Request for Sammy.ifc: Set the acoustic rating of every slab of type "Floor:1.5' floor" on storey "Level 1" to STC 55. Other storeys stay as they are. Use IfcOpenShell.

First a look at what the model holds.

```python
import ifcopenshell
import ifcopenshell.util.element

model = ifcopenshell.open("Sammy.ifc")
print(model.schema)
storey = next(s for s in model.by_type("IfcBuildingStorey") if s.Name == "Level 1")
slabs = [e for e in ifcopenshell.util.element.get_decomposition(storey) if e.is_a("IfcSlab")]
seen = {}
for e in slabs:
    element_type = ifcopenshell.util.element.get_type(e)
    key = (element_type.Name if element_type != e and element_type else None, ifcopenshell.util.element.get_pset(e, "Pset_SlabCommon", "AcousticRating"))
    seen[key] = seen.get(key, 0) + 1
for (name, value), count in sorted(seen.items(), key=str):
    print(count, "x", name, "|", value)
```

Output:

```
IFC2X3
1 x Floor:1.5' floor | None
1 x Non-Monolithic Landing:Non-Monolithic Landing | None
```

```python
import ifcopenshell
import ifcopenshell.api.pset
import ifcopenshell.util.element

model = ifcopenshell.open("Sammy.ifc")

storey = next(s for s in model.by_type("IfcBuildingStorey") if s.Name == "Level 1")
slabs = [e for e in ifcopenshell.util.element.get_decomposition(storey) if e.is_a("IfcSlab")]

count = 0
for e in slabs:
    element_type = ifcopenshell.util.element.get_type(e)
    if element_type in (None, e) or element_type.Name != "Floor:1.5' floor":
        continue
    # add_pset returns the element's existing set when there is one.
    pset = ifcopenshell.api.pset.add_pset(model, product=e, name="Pset_SlabCommon")
    ifcopenshell.api.pset.edit_pset(model, pset=pset, properties={"AcousticRating": "STC 55"})
    count += 1

print(count, "slabs updated")

model.write("Sammy_rev.ifc")
```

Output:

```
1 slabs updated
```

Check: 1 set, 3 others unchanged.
